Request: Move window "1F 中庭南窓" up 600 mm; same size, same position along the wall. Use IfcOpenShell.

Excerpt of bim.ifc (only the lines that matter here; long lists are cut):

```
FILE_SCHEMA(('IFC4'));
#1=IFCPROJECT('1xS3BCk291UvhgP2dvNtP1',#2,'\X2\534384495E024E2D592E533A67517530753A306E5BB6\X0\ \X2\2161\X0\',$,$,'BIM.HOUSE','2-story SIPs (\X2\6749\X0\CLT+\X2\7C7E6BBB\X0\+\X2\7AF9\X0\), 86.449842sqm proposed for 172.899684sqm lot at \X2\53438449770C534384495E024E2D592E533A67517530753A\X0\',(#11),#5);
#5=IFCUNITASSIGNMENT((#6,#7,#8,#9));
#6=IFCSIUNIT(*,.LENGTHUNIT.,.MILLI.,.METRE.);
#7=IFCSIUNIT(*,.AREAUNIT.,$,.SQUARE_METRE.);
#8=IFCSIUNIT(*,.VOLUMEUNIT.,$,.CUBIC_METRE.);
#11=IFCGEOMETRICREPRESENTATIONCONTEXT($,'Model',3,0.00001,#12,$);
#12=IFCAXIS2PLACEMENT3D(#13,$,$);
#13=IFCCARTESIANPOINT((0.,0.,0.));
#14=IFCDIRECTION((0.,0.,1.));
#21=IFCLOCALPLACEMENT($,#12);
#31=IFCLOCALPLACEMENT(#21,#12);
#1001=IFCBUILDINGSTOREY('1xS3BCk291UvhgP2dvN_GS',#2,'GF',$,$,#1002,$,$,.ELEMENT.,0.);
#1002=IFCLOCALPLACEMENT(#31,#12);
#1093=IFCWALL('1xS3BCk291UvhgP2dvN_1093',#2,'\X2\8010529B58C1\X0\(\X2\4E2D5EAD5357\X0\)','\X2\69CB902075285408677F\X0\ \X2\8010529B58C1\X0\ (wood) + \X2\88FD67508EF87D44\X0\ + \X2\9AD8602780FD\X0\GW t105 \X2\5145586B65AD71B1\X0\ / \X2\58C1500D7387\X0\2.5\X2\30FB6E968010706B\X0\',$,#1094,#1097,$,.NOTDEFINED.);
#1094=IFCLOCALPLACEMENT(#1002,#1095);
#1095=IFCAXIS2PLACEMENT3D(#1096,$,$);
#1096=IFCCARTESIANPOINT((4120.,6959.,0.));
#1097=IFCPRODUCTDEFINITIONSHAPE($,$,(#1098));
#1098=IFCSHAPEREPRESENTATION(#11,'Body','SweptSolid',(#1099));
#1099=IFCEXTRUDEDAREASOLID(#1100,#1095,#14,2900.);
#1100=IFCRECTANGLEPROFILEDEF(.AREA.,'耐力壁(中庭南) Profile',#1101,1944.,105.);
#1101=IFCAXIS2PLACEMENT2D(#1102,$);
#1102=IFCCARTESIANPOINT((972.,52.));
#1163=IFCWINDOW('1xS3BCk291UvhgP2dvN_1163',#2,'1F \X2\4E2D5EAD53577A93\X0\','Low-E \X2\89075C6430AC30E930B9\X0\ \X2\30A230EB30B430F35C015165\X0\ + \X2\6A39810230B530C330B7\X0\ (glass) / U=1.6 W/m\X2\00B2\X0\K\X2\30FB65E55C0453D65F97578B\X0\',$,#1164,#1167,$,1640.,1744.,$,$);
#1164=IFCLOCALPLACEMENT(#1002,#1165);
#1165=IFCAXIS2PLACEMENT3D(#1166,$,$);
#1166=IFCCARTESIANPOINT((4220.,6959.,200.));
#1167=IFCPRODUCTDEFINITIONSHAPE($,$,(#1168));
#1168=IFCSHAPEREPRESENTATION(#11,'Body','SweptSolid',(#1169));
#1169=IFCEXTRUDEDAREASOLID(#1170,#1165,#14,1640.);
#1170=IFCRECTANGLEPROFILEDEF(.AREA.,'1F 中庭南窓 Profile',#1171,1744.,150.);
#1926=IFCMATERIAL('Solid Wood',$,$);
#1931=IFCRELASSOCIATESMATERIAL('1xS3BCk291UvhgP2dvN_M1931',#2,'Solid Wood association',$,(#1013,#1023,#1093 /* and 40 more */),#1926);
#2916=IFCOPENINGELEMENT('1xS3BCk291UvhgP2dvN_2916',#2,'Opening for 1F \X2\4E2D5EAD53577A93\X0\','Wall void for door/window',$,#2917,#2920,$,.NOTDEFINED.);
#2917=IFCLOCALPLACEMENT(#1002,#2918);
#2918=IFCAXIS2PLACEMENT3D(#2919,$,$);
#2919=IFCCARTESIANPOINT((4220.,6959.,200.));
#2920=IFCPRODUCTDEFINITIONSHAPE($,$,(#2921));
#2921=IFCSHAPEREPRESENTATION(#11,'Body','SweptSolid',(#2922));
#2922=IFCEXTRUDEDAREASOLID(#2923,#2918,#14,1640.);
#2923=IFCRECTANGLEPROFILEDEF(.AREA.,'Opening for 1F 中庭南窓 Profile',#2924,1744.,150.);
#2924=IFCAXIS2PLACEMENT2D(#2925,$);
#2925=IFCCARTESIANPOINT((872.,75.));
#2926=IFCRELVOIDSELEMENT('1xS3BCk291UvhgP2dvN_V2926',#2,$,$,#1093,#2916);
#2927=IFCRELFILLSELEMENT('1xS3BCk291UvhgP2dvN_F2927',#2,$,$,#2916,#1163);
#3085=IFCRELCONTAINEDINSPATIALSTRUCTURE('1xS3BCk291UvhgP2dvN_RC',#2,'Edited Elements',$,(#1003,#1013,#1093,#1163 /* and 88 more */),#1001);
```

```python
import numpy as np
import ifcopenshell
import ifcopenshell.api.geometry
import ifcopenshell.util.placement
import ifcopenshell.util.unit

model = ifcopenshell.open("bim.ifc")
unit_scale = ifcopenshell.util.unit.calculate_unit_scale(model)

window = model.by_id(1163)
opening = window.FillsVoids[0].RelatingOpeningElement
dz = 0.6 / unit_scale

shift = np.array([0.0, 0.0, dz])
# The window is not placed relative to its opening, so move both.
for product in (opening, window):
    matrix = ifcopenshell.util.placement.get_local_placement(product.ObjectPlacement)
    matrix[:3, 3] += shift
    ifcopenshell.api.geometry.edit_object_placement(model, product=product, matrix=matrix, is_si=False)

print(f"moved by {dz * unit_scale:+.3f} m")

model.write("bim_edited.ifc")
```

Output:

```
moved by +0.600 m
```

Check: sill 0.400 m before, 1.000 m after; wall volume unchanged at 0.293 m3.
